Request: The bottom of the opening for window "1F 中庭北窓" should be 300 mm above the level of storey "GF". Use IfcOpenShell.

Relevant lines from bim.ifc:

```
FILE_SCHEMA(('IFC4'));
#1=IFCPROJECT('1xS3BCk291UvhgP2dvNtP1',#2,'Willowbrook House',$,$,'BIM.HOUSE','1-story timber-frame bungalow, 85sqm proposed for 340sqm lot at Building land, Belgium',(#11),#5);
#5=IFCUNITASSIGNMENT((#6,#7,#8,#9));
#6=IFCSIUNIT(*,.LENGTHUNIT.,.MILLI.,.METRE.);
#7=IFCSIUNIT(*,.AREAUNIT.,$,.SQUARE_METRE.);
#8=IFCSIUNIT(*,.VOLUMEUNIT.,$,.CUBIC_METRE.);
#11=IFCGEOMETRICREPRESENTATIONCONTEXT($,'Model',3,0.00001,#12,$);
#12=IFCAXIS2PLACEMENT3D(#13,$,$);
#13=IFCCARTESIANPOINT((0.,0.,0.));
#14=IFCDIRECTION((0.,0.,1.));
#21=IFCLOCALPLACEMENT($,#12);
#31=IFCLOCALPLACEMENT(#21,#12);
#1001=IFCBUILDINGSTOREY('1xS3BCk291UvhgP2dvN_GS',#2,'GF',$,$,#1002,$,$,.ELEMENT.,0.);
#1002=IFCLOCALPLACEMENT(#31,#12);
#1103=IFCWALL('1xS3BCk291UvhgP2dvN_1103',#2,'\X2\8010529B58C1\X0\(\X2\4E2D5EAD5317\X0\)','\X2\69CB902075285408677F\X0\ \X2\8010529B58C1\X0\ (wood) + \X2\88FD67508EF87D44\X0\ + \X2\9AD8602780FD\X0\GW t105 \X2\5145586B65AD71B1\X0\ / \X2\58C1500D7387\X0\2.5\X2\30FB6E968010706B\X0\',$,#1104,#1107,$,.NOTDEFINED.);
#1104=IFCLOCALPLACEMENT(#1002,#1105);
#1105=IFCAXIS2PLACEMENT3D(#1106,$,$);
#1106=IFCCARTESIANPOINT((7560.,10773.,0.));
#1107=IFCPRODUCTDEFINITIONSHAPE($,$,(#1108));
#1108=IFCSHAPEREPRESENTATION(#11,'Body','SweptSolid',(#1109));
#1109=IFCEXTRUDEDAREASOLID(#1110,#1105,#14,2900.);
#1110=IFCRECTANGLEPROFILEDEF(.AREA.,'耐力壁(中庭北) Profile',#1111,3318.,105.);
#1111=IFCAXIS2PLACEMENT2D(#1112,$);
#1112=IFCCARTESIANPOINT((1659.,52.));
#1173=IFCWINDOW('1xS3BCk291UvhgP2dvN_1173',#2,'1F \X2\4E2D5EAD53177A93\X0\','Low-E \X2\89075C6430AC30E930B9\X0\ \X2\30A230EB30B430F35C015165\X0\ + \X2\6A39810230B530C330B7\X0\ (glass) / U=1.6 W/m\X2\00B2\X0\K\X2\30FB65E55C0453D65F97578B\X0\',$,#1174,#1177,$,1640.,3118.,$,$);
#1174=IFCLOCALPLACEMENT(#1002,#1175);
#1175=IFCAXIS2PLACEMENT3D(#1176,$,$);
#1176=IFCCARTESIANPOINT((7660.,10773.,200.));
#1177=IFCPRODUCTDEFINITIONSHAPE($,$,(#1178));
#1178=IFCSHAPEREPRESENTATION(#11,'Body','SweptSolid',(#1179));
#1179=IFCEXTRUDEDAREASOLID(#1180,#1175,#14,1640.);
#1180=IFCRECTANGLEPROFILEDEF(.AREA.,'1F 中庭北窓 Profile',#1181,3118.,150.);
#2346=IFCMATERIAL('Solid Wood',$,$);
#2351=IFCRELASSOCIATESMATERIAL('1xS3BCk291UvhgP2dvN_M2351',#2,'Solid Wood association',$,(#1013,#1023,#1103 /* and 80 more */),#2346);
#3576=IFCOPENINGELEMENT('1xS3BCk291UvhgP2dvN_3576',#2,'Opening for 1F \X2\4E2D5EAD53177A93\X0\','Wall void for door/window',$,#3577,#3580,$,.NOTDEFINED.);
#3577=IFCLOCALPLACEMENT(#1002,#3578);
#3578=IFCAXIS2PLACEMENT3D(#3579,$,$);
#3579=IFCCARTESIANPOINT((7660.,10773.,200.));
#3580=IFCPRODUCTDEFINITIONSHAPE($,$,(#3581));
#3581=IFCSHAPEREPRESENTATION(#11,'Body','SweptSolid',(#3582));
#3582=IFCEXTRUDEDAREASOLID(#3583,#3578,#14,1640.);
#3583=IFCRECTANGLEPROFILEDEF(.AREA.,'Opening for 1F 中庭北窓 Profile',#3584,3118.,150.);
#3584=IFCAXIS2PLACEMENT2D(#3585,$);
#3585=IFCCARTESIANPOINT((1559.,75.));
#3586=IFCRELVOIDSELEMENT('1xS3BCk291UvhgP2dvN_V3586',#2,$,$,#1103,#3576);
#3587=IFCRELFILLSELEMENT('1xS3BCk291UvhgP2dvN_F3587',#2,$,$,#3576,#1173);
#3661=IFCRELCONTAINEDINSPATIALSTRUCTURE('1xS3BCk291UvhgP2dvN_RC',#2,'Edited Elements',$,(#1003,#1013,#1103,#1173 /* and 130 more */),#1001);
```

```python
import numpy as np
import ifcopenshell
import ifcopenshell.api.geometry
import ifcopenshell.geom
import ifcopenshell.util.element
import ifcopenshell.util.placement
import ifcopenshell.util.shape
import ifcopenshell.util.unit

model = ifcopenshell.open("bim.ifc")
unit_scale = ifcopenshell.util.unit.calculate_unit_scale(model)

window = model.by_guid("1xS3BCk291UvhgP2dvN_1173")
opening = window.FillsVoids[0].RelatingOpeningElement
storey = ifcopenshell.util.element.get_container(window, ifc_class="IfcBuildingStorey")
level = ifcopenshell.util.placement.get_local_placement(storey.ObjectPlacement)[2, 3]

# The opening's origin need not be at the sill, so measure its lowest point.
shape = ifcopenshell.geom.create_shape(ifcopenshell.geom.settings(), opening)
bottom = ifcopenshell.util.shape.get_shape_bottom_elevation(shape, shape.geometry) / unit_scale
dz = level + 300.0 - bottom

shift = np.array([0.0, 0.0, dz])
# The window is not placed relative to its opening, so move both.
for product in (opening, window):
    matrix = ifcopenshell.util.placement.get_local_placement(product.ObjectPlacement)
    matrix[:3, 3] += shift
    ifcopenshell.api.geometry.edit_object_placement(model, product=product, matrix=matrix, is_si=False)

print(f"moved by {dz * unit_scale:+.3f} m")

model.write("bim_rev.ifc")
```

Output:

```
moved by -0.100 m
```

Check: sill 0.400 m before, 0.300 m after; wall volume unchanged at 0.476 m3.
